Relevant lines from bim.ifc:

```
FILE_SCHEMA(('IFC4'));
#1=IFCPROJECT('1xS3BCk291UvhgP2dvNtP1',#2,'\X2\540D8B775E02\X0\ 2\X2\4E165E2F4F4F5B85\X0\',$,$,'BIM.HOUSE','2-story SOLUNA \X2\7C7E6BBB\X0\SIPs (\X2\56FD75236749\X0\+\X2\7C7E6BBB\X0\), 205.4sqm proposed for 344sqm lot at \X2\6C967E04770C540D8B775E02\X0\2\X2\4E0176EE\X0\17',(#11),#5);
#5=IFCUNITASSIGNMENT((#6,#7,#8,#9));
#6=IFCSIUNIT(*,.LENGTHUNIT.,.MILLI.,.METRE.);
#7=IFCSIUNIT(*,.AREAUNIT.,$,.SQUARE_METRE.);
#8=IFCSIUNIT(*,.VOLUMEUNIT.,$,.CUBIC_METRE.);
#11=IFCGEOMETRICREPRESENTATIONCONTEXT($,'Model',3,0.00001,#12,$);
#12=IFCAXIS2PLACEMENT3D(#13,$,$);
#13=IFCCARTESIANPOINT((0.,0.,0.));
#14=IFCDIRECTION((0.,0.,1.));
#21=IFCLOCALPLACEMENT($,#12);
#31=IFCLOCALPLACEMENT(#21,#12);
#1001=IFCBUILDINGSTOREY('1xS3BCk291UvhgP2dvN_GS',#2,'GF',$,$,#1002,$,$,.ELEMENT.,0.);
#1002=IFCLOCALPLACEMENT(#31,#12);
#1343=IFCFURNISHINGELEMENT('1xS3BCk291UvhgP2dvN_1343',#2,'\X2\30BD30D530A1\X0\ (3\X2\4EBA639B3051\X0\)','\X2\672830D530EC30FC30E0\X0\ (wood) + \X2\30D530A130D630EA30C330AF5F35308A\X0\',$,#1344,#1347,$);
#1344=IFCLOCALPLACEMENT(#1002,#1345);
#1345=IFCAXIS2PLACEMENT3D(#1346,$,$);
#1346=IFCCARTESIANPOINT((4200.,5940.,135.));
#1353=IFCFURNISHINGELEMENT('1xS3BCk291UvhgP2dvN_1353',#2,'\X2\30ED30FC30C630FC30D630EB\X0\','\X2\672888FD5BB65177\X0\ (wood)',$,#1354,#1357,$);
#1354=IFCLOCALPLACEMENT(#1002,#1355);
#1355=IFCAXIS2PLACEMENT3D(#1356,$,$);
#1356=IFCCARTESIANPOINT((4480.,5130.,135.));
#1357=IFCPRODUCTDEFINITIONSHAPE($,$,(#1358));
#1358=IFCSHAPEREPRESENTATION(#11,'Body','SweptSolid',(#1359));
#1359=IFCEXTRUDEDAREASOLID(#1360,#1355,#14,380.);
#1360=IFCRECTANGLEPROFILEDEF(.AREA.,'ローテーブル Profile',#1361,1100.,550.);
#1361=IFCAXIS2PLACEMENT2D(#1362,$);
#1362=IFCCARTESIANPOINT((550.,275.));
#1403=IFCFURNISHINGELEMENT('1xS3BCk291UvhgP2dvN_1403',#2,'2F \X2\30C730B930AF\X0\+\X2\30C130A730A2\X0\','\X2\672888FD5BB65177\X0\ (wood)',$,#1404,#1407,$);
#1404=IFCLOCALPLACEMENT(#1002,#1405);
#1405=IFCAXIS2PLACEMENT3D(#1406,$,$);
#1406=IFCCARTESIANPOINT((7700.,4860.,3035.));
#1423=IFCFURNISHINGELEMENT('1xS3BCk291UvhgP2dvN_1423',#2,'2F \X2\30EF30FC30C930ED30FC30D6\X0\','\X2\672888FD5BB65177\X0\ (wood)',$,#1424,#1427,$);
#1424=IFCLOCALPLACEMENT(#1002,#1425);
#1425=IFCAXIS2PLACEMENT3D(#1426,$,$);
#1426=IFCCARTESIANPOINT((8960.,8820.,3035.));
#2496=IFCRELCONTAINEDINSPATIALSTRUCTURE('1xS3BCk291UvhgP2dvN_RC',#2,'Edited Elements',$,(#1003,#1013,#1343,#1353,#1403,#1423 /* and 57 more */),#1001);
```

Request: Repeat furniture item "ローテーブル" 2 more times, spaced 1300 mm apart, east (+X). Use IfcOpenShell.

```python
import numpy as np
import ifcopenshell
import ifcopenshell.api.geometry
import ifcopenshell.api.root
import ifcopenshell.util.element
import ifcopenshell.util.placement
import ifcopenshell.util.unit

model = ifcopenshell.open("bim.ifc")
unit_scale = ifcopenshell.util.unit.calculate_unit_scale(model)


def reuse_history(source, copy):
    """copy_class also copies each property set's owner history, people and application; keep the originals."""
    for rel in copy.IsDefinedBy:
        if rel.is_a("IfcRelDefinesByProperties") and (history := rel.RelatingPropertyDefinition.OwnerHistory):
            rel.RelatingPropertyDefinition.OwnerHistory = source.OwnerHistory
            ifcopenshell.util.element.remove_deep2(model, history)


source = model.by_id(1353)
base = ifcopenshell.util.placement.get_local_placement(source.ObjectPlacement)
step = np.array([1.0, 0.0, 0.0]) * 1.3 / unit_scale

for i in range(1, 3):
    copy = ifcopenshell.api.root.copy_class(model, product=source)
    copy.Representation = ifcopenshell.util.element.copy_deep(
        model, source.Representation, exclude=["IfcGeometricRepresentationContext", "IfcRepresentationMap"]
    )
    reuse_history(source, copy)
    matrix = base.copy()
    matrix[:3, 3] += i * step
    print("added at", matrix[:3, 3].round(3) + 0.0)
    ifcopenshell.api.geometry.edit_object_placement(model, product=copy, matrix=matrix, is_si=False)

model.write("bim_rev.ifc")
```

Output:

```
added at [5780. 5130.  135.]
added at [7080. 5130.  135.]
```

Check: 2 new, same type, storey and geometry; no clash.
